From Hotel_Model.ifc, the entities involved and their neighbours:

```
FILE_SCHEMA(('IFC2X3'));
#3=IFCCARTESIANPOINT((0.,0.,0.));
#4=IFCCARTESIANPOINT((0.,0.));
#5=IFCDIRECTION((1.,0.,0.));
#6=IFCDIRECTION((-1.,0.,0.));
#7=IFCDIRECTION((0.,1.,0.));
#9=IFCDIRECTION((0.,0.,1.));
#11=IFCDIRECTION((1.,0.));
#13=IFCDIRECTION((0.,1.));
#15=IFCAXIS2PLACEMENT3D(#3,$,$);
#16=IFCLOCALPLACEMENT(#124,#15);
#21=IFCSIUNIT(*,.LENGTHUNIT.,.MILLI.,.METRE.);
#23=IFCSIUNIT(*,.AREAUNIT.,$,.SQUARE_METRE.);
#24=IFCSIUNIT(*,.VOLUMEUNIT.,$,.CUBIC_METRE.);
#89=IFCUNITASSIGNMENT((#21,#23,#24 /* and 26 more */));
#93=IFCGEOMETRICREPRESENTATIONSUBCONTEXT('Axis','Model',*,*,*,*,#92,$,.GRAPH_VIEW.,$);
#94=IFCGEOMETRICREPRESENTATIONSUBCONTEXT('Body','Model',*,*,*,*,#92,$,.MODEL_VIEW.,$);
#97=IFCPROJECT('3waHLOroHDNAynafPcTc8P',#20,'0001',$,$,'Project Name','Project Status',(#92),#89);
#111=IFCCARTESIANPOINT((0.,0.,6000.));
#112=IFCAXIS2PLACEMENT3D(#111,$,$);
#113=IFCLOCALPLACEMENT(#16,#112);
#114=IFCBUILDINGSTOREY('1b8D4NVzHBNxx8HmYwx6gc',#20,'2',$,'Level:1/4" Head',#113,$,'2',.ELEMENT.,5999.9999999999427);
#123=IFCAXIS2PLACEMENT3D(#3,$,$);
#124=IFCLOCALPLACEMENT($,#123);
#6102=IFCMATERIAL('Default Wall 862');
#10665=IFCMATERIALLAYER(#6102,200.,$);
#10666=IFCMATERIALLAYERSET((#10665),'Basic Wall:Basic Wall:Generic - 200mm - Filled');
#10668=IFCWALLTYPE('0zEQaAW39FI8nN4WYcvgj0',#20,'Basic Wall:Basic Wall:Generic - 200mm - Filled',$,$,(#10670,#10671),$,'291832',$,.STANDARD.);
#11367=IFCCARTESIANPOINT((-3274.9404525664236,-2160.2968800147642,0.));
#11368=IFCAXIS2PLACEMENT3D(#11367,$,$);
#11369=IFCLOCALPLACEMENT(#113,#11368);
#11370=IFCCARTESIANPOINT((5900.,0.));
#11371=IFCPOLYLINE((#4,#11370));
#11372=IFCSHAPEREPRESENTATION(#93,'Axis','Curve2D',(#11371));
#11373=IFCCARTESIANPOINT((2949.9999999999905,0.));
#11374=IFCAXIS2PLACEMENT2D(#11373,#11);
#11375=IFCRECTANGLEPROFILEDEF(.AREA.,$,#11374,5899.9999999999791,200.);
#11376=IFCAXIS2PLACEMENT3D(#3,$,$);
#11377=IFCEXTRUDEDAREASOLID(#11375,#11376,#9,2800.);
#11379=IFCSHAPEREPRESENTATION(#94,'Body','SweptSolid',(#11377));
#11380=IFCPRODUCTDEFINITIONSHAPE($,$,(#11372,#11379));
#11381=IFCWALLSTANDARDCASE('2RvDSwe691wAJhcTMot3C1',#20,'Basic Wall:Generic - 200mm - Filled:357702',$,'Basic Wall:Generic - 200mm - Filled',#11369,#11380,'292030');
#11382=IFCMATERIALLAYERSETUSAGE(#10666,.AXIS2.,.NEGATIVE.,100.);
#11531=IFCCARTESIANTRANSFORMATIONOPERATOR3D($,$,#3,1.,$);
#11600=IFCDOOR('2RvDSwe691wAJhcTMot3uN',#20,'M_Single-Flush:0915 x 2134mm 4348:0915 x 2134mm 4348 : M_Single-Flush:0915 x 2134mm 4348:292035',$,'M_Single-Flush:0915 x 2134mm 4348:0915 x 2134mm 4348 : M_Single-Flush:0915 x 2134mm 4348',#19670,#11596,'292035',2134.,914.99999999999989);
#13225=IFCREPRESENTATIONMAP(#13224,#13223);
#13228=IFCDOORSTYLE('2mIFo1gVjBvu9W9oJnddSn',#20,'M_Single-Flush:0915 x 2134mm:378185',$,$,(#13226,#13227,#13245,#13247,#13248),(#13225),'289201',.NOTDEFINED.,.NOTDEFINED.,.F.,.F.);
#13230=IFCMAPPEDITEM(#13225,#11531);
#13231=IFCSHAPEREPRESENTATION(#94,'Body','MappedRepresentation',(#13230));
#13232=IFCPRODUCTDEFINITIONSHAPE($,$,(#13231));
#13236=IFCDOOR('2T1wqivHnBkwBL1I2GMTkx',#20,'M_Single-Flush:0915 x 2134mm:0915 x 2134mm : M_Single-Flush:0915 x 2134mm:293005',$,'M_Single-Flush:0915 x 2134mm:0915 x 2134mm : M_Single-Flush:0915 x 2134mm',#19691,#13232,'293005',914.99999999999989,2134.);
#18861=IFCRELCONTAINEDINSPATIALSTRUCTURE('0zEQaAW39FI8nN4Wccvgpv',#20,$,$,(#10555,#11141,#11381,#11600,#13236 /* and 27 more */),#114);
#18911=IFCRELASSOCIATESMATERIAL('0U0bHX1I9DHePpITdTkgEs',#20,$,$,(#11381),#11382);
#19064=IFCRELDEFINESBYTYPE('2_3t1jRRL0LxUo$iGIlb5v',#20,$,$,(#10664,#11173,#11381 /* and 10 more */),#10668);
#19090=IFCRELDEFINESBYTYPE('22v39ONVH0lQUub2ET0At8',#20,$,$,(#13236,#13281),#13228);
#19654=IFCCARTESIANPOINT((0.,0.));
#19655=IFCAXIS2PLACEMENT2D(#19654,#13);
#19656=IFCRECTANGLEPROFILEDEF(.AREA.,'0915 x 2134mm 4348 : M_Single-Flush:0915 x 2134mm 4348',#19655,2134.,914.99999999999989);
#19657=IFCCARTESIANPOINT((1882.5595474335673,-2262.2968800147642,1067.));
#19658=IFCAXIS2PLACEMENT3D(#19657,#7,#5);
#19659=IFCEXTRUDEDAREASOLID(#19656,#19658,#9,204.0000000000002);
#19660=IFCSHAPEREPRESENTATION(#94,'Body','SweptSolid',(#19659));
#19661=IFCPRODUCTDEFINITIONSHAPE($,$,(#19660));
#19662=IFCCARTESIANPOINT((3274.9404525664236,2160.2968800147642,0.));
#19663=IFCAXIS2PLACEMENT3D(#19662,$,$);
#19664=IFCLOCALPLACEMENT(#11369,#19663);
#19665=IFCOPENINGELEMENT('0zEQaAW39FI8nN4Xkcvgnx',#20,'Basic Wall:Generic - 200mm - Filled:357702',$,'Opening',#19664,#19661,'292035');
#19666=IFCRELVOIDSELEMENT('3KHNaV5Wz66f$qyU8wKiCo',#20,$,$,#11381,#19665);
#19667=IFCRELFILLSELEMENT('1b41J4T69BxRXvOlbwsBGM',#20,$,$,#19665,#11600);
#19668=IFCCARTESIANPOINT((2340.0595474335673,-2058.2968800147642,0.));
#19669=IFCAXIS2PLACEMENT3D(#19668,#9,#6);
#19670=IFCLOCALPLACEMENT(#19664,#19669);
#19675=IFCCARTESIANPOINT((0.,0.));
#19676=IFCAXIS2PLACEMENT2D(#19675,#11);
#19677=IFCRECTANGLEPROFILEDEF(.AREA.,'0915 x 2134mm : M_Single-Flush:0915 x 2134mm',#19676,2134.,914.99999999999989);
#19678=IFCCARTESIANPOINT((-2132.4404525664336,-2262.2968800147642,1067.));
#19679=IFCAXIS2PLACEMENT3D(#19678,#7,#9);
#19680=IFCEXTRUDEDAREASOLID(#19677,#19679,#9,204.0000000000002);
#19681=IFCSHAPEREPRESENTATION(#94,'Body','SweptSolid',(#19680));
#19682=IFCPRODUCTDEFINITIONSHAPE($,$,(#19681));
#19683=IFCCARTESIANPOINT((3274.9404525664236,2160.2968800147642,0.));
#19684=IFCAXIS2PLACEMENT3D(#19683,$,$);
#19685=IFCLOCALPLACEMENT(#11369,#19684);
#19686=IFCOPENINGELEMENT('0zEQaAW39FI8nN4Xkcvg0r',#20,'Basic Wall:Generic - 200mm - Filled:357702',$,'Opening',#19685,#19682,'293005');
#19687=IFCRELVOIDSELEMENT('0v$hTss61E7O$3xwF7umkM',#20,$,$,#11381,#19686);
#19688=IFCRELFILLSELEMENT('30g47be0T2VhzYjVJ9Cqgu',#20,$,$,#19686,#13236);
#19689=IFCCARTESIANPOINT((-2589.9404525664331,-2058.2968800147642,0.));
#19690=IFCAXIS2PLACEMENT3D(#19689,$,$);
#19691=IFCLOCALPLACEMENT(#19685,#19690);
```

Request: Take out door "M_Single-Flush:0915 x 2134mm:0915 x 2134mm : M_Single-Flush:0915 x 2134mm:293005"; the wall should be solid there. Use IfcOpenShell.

```python
import ifcopenshell
import ifcopenshell.api.feature
import ifcopenshell.api.root
import ifcopenshell.geom
import ifcopenshell.util.shape

model = ifcopenshell.open("Hotel_Model.ifc")
settings = ifcopenshell.geom.settings()


def volume(element):
    """Net volume in cubic metres, openings subtracted."""
    shape = ifcopenshell.geom.create_shape(settings, element)
    return ifcopenshell.util.shape.get_volume(shape.geometry)


door = model.by_id(13236)
opening = door.FillsVoids[0].RelatingOpeningElement
wall = opening.VoidsElements[0].RelatingBuildingElement
before = volume(wall)

ifcopenshell.api.root.remove_product(model, product=door)
ifcopenshell.api.feature.remove_feature(model, feature=opening)

after = volume(wall)

print(f"wall volume {before:.3f} -> {after:.3f} m3")

model.write("Hotel_Model_edited.ifc")
```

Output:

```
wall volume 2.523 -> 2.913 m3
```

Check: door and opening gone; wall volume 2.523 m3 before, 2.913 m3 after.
